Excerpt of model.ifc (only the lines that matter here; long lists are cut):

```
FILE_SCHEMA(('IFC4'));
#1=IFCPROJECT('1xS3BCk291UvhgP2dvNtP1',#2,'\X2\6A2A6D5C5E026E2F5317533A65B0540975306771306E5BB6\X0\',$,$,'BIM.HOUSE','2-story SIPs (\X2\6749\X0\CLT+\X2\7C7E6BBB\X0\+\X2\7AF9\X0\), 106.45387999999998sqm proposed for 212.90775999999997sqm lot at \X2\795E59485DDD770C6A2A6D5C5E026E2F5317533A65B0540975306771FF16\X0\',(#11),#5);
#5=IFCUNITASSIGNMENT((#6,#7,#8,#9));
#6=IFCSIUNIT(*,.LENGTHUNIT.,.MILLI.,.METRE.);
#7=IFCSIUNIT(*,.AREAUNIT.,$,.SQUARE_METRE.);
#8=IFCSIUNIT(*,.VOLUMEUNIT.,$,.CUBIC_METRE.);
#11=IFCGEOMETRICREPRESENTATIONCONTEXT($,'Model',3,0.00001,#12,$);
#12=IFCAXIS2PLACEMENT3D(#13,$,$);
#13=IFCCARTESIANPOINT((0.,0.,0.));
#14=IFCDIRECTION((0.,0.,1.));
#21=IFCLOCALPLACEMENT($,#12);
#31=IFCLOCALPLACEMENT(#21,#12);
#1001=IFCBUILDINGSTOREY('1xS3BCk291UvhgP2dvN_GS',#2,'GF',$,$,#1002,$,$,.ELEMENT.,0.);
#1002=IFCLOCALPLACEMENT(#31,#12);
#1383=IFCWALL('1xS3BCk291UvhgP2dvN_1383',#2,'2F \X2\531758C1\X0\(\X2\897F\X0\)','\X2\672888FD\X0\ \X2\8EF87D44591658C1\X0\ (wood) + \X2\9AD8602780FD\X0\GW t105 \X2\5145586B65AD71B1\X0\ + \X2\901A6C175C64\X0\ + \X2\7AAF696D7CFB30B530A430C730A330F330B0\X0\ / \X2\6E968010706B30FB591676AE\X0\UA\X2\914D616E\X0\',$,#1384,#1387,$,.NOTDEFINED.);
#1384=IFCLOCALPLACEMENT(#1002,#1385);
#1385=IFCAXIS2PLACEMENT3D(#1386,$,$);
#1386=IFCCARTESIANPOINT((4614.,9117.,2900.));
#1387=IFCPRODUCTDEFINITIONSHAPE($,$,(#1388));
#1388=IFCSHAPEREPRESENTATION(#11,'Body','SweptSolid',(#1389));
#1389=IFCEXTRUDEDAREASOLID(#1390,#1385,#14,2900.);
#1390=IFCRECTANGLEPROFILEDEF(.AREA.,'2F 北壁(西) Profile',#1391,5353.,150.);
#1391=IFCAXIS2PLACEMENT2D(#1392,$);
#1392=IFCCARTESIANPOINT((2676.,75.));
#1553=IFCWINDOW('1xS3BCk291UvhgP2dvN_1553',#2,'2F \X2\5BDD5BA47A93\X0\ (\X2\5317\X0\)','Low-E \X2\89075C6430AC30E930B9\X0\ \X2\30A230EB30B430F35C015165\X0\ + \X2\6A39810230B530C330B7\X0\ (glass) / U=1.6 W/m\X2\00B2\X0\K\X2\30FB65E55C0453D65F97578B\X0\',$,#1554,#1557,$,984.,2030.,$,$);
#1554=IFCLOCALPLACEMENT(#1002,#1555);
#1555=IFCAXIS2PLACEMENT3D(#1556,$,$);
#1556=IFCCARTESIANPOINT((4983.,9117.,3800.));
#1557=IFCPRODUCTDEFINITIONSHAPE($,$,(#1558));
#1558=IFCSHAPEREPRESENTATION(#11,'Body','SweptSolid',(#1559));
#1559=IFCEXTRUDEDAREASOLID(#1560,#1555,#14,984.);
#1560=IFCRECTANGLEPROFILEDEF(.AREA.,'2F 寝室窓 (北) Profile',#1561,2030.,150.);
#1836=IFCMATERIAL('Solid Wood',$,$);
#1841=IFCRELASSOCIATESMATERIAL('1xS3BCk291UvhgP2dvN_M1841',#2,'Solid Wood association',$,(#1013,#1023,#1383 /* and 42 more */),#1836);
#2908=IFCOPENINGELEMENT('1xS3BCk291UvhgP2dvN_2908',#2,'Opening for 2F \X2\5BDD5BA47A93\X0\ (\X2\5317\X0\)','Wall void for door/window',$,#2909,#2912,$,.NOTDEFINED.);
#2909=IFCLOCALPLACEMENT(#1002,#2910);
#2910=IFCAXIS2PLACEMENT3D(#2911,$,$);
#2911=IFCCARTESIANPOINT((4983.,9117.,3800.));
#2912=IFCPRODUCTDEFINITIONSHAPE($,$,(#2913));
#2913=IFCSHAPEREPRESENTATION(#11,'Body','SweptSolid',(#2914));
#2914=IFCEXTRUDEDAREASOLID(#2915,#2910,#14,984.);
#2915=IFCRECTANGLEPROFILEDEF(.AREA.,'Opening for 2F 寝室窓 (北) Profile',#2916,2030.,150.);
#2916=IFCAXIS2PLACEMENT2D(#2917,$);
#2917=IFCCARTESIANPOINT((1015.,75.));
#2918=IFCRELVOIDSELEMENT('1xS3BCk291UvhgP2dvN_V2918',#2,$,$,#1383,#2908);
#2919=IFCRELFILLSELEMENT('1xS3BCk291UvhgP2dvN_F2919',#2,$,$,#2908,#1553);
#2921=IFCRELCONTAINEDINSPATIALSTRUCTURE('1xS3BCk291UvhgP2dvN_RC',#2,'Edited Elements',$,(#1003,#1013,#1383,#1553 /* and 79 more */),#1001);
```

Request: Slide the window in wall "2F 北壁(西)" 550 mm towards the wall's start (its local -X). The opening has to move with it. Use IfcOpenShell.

```python
import ifcopenshell
import ifcopenshell.api.geometry
import ifcopenshell.util.placement
import ifcopenshell.util.unit

model = ifcopenshell.open("model.ifc")
unit_scale = ifcopenshell.util.unit.calculate_unit_scale(model)

window = model.by_guid("1xS3BCk291UvhgP2dvN_1553")
opening = window.FillsVoids[0].RelatingOpeningElement
wall = opening.VoidsElements[0].RelatingBuildingElement

wall_matrix = ifcopenshell.util.placement.get_local_placement(wall.ObjectPlacement)
shift = wall_matrix[:3, 0] * -0.55 / unit_scale
before = ifcopenshell.util.placement.get_local_placement(window.ObjectPlacement)[:3, 3].copy()

# The window is not placed relative to its opening, so move both.
for product in (opening, window):
    matrix = ifcopenshell.util.placement.get_local_placement(product.ObjectPlacement)
    matrix[:3, 3] += shift
    ifcopenshell.api.geometry.edit_object_placement(model, product=product, matrix=matrix, is_si=False)

after = ifcopenshell.util.placement.get_local_placement(window.ObjectPlacement)[:3, 3]
print("window moved by", (after - before).round(3) + 0.0)

model.write("model_v2.ifc")
```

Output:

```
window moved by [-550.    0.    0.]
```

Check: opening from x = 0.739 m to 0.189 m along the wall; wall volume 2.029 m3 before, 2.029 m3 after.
